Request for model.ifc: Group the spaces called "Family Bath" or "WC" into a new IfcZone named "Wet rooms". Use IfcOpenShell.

First a look at what the model holds.

```python
import ifcopenshell

model = ifcopenshell.open("model.ifc")
print(model.schema)
seen = {}
for space in model.by_type("IfcSpace"):
    seen[space.LongName] = seen.get(space.LongName, 0) + 1
for name, count in sorted(seen.items(), key=str):
    print(count, "x", name)
print("zones:", [z.Name for z in model.by_type("IfcZone")][:20])
```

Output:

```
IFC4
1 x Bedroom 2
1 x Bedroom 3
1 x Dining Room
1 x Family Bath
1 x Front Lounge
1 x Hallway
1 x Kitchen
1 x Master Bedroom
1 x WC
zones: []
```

```python
import ifcopenshell
import ifcopenshell.api.group
import ifcopenshell.api.root

model = ifcopenshell.open("model.ifc")

names = {"Family Bath", "WC"}
spaces = [s for s in model.by_type("IfcSpace") if s.LongName in names]

zone = ifcopenshell.api.root.create_entity(model, ifc_class="IfcZone", name="Wet rooms")
ifcopenshell.api.group.assign_group(model, products=spaces, group=zone)
print(len(spaces), "spaces in", zone.Name)

model.write("model_rev.ifc")
```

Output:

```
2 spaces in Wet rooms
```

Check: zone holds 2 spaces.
